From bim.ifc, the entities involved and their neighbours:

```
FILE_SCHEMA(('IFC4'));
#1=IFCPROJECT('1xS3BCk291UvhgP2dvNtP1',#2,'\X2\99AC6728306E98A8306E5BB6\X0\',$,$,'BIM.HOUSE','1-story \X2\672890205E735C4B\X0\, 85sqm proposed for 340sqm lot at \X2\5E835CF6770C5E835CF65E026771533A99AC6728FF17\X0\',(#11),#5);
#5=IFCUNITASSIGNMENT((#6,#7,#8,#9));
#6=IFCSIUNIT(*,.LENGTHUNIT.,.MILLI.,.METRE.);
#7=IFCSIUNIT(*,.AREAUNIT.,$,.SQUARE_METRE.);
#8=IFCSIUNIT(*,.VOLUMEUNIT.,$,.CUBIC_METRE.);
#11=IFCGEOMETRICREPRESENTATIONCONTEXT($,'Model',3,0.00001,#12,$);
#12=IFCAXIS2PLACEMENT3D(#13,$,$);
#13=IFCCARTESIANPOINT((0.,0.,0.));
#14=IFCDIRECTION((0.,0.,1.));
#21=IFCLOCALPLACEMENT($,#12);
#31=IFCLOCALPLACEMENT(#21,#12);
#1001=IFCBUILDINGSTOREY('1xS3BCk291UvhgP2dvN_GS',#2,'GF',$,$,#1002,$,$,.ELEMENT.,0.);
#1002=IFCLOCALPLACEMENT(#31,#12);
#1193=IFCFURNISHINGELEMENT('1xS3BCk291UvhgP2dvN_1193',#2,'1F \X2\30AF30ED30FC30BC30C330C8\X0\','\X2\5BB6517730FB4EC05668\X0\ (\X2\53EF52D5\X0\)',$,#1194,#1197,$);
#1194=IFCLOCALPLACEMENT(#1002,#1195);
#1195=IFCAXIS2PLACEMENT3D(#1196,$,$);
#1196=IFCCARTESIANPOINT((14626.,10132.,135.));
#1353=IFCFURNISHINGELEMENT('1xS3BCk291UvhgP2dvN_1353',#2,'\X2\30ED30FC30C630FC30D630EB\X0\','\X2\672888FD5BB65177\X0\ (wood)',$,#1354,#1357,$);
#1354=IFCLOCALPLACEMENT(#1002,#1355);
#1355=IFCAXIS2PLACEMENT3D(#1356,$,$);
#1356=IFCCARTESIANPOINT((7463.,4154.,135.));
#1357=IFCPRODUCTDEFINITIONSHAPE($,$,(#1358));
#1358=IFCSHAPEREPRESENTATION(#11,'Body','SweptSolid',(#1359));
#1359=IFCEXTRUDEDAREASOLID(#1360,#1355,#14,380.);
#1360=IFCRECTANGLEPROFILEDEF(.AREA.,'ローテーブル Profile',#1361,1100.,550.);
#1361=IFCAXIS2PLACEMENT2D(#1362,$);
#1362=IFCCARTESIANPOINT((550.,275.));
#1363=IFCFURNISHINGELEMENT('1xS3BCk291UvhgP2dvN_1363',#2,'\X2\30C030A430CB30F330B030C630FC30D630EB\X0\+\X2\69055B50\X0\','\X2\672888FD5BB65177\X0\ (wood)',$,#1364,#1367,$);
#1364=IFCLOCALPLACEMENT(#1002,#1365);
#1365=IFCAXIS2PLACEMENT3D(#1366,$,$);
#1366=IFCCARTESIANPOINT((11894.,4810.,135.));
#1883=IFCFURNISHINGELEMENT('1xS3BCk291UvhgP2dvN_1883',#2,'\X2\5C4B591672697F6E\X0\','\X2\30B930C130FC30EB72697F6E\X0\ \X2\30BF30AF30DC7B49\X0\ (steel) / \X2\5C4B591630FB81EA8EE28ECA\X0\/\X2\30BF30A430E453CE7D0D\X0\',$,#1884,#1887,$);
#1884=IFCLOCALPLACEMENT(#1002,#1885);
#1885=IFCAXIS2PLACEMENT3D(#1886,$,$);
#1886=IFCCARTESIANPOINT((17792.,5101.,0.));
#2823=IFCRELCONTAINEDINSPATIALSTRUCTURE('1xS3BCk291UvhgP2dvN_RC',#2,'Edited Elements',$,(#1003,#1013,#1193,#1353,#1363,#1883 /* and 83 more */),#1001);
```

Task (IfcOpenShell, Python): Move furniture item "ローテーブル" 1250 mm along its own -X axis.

```python
import ifcopenshell
import ifcopenshell.api.geometry
import ifcopenshell.util.placement
import ifcopenshell.util.unit

model = ifcopenshell.open("bim.ifc")
unit_scale = ifcopenshell.util.unit.calculate_unit_scale(model)

item = model.by_guid("1xS3BCk291UvhgP2dvN_1353")
matrix = ifcopenshell.util.placement.get_local_placement(item.ObjectPlacement)
matrix[:3, 3] -= matrix[:3, 0] * 1.25 / unit_scale
ifcopenshell.api.geometry.edit_object_placement(model, product=item, matrix=matrix, is_si=False)

print(ifcopenshell.util.placement.get_local_placement(item.ObjectPlacement).round(3) + 0.0)

model.write("bim-out.ifc")
```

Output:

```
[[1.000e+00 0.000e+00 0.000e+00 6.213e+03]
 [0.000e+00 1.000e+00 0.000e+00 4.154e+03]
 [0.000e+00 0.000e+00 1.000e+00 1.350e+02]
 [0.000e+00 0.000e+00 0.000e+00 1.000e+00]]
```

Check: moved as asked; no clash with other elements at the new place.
